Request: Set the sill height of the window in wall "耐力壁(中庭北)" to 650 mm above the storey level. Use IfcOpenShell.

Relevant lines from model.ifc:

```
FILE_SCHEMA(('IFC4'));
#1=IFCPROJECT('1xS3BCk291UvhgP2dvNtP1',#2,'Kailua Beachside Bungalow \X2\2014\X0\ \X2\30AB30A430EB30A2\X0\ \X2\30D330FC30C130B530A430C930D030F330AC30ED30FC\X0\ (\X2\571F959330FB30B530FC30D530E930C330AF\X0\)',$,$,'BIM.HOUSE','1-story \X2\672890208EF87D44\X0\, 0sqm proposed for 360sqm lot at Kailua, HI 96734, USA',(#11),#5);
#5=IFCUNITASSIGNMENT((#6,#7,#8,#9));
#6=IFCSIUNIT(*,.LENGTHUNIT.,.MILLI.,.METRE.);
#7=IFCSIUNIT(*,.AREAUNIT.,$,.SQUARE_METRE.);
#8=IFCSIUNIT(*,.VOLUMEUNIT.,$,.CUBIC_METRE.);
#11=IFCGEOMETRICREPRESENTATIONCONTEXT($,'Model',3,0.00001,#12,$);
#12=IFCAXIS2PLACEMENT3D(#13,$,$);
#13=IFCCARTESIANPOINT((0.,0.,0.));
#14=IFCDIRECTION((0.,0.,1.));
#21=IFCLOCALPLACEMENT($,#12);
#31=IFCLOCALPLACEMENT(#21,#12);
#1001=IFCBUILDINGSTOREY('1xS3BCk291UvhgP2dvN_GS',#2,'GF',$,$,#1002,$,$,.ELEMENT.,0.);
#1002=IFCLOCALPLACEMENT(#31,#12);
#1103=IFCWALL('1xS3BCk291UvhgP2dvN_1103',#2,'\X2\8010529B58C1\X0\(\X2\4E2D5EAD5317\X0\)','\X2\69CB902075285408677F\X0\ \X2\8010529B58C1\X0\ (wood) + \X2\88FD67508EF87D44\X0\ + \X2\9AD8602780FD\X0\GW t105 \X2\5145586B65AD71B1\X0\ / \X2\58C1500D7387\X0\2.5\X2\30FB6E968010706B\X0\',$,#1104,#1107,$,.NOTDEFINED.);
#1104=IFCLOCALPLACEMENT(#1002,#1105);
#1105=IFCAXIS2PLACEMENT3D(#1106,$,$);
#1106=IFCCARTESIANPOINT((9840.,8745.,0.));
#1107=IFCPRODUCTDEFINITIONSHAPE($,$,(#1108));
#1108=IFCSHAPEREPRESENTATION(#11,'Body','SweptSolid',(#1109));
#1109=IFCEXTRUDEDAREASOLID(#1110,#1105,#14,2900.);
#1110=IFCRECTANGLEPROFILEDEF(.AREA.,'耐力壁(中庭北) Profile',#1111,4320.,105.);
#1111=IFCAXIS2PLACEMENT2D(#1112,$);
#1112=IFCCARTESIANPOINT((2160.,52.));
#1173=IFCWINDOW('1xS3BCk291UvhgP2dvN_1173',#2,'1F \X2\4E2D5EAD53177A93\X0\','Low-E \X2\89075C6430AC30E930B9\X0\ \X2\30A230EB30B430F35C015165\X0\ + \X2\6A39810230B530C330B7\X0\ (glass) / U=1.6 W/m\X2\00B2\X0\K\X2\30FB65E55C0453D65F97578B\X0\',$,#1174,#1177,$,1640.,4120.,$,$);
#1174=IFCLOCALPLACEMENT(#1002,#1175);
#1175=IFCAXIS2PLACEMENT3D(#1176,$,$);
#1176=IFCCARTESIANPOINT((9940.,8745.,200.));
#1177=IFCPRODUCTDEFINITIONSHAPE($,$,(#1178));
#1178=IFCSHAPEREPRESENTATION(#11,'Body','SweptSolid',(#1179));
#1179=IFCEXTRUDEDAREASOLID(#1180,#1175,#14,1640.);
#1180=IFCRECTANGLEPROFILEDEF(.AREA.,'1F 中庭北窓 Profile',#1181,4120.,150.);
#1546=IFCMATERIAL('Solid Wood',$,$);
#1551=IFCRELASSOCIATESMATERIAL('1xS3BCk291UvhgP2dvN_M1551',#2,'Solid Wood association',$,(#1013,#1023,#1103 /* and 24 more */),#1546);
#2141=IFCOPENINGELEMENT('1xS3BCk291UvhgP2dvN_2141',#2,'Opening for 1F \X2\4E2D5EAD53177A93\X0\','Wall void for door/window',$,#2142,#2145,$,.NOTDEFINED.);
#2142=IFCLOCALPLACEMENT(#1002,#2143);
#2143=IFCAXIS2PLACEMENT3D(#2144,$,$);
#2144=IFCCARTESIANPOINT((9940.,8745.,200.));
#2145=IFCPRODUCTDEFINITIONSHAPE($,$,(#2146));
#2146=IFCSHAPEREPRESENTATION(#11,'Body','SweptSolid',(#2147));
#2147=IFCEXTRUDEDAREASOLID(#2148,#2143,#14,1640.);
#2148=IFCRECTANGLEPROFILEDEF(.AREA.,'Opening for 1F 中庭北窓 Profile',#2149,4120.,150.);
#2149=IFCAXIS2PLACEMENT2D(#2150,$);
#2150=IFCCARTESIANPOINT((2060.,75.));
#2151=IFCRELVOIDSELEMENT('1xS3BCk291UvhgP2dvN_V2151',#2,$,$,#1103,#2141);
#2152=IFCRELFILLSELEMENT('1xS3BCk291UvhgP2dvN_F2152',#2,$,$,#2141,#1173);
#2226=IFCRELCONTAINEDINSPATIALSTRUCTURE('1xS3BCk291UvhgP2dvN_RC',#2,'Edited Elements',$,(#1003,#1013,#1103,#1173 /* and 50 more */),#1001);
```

```python
import numpy as np
import ifcopenshell
import ifcopenshell.api.geometry
import ifcopenshell.geom
import ifcopenshell.util.element
import ifcopenshell.util.placement
import ifcopenshell.util.shape
import ifcopenshell.util.unit

model = ifcopenshell.open("model.ifc")
unit_scale = ifcopenshell.util.unit.calculate_unit_scale(model)

window = model.by_id(1173)
opening = window.FillsVoids[0].RelatingOpeningElement
storey = ifcopenshell.util.element.get_container(window, ifc_class="IfcBuildingStorey")
level = ifcopenshell.util.placement.get_local_placement(storey.ObjectPlacement)[2, 3]

# The opening's origin need not be at the sill, so measure its lowest point.
shape = ifcopenshell.geom.create_shape(ifcopenshell.geom.settings(), opening)
bottom = ifcopenshell.util.shape.get_shape_bottom_elevation(shape, shape.geometry) / unit_scale
dz = level + 650.0 - bottom

shift = np.array([0.0, 0.0, dz])
# The window is not placed relative to its opening, so move both.
for product in (opening, window):
    matrix = ifcopenshell.util.placement.get_local_placement(product.ObjectPlacement)
    matrix[:3, 3] += shift
    ifcopenshell.api.geometry.edit_object_placement(model, product=product, matrix=matrix, is_si=False)

print(f"moved by {dz * unit_scale:+.3f} m")

model.write("model_v2.ifc")
```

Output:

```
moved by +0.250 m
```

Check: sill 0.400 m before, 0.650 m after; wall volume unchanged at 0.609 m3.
